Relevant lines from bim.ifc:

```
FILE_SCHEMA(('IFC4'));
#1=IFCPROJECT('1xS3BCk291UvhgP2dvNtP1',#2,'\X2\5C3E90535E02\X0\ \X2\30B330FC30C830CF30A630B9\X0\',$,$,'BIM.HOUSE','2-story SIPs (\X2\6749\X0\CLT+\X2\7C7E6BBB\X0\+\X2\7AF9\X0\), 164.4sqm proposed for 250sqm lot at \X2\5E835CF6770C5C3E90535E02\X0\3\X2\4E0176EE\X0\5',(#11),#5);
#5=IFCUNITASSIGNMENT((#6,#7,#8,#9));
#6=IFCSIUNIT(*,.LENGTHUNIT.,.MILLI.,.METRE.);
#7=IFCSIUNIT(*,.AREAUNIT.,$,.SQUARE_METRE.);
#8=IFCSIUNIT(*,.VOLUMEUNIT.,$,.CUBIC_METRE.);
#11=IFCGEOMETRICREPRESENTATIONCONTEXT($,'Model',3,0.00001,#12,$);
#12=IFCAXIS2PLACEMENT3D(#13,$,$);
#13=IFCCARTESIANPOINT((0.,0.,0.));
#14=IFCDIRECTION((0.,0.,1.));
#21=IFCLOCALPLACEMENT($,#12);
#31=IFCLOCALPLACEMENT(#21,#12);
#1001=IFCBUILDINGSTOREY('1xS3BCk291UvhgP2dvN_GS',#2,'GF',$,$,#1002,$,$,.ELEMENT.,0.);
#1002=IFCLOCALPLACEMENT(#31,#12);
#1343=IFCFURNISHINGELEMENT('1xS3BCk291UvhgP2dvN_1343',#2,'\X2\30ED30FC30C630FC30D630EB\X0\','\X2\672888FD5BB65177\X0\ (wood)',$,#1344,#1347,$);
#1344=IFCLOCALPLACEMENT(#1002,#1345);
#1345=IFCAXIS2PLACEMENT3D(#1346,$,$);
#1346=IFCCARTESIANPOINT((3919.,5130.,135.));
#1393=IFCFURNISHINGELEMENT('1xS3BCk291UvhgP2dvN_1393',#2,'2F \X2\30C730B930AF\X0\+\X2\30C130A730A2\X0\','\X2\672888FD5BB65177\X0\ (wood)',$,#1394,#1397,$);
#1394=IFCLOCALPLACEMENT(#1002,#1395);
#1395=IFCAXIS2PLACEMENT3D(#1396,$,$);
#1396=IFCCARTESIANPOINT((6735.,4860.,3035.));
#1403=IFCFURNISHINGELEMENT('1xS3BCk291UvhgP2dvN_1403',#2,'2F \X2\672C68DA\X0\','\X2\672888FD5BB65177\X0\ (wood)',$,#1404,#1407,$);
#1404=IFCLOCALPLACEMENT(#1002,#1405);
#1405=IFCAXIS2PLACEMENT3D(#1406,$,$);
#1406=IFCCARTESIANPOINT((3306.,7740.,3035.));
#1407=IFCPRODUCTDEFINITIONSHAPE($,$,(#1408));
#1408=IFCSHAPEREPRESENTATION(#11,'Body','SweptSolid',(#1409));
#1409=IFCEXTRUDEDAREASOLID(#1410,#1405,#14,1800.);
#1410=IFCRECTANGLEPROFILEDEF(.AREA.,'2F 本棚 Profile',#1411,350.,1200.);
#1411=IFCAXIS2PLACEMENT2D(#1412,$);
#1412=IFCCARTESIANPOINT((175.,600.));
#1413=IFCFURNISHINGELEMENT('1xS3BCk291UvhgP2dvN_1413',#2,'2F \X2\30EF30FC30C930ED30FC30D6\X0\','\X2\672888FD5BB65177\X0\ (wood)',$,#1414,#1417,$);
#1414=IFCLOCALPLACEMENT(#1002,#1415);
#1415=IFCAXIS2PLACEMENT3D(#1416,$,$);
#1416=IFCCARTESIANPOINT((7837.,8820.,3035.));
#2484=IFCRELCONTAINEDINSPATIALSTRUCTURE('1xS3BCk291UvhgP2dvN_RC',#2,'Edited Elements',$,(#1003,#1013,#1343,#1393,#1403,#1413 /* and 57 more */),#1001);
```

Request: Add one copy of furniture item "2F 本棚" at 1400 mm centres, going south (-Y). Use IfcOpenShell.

```python
import numpy as np
import ifcopenshell
import ifcopenshell.api.geometry
import ifcopenshell.api.root
import ifcopenshell.util.element
import ifcopenshell.util.placement
import ifcopenshell.util.unit

model = ifcopenshell.open("bim.ifc")
unit_scale = ifcopenshell.util.unit.calculate_unit_scale(model)


def reuse_history(source, copy):
    """copy_class also copies each property set's owner history, people and application; keep the originals."""
    for rel in copy.IsDefinedBy:
        if rel.is_a("IfcRelDefinesByProperties") and (history := rel.RelatingPropertyDefinition.OwnerHistory):
            rel.RelatingPropertyDefinition.OwnerHistory = source.OwnerHistory
            ifcopenshell.util.element.remove_deep2(model, history)


source = model.by_guid("1xS3BCk291UvhgP2dvN_1403")
base = ifcopenshell.util.placement.get_local_placement(source.ObjectPlacement)
step = np.array([0.0, -1.0, 0.0]) * 1.4 / unit_scale

for i in range(1, 2):
    copy = ifcopenshell.api.root.copy_class(model, product=source)
    copy.Representation = ifcopenshell.util.element.copy_deep(
        model, source.Representation, exclude=["IfcGeometricRepresentationContext", "IfcRepresentationMap"]
    )
    reuse_history(source, copy)
    matrix = base.copy()
    matrix[:3, 3] += i * step
    print("added at", matrix[:3, 3].round(3) + 0.0)
    ifcopenshell.api.geometry.edit_object_placement(model, product=copy, matrix=matrix, is_si=False)

model.write("bim_rev.ifc")
```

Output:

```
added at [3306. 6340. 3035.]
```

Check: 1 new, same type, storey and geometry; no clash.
